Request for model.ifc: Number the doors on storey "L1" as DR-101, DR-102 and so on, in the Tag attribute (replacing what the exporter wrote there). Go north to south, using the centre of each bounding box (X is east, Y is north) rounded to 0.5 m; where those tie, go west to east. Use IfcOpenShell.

First a look at what the model holds.

```python
import ifcopenshell
import ifcopenshell.util.element
import ifcopenshell.util.placement

model = ifcopenshell.open("model.ifc")
print(model.schema)
storey = next(s for s in model.by_type("IfcBuildingStorey") if s.Name == "L1")
doors = [e for e in ifcopenshell.util.element.get_decomposition(storey) if e.is_a("IfcDoor")]
for e in sorted(doors, key=lambda e: e.id()):
    origin = ifcopenshell.util.placement.get_local_placement(e.ObjectPlacement)[:3, 3]
    print(e.id(), e.Tag, e.Name, origin.round(2) + 0.0, sep=" | ")
```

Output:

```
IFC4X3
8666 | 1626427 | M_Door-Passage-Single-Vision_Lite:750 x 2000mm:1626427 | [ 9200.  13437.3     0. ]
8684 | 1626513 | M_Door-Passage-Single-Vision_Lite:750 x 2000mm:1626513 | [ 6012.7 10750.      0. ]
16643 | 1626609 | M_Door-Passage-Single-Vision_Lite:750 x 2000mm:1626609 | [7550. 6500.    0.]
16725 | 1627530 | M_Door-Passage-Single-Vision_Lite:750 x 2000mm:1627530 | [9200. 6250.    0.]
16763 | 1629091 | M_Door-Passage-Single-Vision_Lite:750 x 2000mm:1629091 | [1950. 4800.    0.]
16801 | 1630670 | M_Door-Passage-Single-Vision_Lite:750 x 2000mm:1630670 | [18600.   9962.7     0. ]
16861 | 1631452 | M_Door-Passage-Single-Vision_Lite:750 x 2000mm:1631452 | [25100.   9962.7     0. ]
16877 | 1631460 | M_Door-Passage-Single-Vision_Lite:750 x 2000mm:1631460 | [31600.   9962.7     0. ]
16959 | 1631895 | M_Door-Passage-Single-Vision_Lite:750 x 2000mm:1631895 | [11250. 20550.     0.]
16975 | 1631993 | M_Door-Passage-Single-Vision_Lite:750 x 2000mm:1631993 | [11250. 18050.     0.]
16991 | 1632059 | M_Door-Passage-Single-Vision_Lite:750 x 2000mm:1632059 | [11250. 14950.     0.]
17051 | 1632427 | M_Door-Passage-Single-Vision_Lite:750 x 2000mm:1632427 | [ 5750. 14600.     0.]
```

```python
import ifcopenshell
import ifcopenshell.geom
import ifcopenshell.util.element
import ifcopenshell.util.shape

model = ifcopenshell.open("model.ifc")
settings = ifcopenshell.geom.settings()
settings.set("use-world-coords", True)


def centre(element):
    shape = ifcopenshell.geom.create_shape(settings, element)
    return ifcopenshell.util.shape.get_bbox_centroid(shape.geometry)


storey = next(s for s in model.by_type("IfcBuildingStorey") if s.Name == "L1")
doors = [e for e in ifcopenshell.util.element.get_decomposition(storey) if e.is_a("IfcDoor")]

# Insertion points can sit at a corner or the storey origin, so sort by the geometry (in metres).
centres = {e: centre(e) for e in doors}
doors.sort(key=lambda e: (-round(centres[e][1] / 0.5), centres[e][0]))

for i, e in enumerate(doors, start=1):
    number = f"DR-1{i:02d}"
    e.Tag = number
    print(e.id(), number)

model.write("model_v2.ifc")
```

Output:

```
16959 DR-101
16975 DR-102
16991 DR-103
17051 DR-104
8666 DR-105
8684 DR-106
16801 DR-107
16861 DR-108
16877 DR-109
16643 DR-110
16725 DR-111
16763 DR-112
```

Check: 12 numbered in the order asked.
